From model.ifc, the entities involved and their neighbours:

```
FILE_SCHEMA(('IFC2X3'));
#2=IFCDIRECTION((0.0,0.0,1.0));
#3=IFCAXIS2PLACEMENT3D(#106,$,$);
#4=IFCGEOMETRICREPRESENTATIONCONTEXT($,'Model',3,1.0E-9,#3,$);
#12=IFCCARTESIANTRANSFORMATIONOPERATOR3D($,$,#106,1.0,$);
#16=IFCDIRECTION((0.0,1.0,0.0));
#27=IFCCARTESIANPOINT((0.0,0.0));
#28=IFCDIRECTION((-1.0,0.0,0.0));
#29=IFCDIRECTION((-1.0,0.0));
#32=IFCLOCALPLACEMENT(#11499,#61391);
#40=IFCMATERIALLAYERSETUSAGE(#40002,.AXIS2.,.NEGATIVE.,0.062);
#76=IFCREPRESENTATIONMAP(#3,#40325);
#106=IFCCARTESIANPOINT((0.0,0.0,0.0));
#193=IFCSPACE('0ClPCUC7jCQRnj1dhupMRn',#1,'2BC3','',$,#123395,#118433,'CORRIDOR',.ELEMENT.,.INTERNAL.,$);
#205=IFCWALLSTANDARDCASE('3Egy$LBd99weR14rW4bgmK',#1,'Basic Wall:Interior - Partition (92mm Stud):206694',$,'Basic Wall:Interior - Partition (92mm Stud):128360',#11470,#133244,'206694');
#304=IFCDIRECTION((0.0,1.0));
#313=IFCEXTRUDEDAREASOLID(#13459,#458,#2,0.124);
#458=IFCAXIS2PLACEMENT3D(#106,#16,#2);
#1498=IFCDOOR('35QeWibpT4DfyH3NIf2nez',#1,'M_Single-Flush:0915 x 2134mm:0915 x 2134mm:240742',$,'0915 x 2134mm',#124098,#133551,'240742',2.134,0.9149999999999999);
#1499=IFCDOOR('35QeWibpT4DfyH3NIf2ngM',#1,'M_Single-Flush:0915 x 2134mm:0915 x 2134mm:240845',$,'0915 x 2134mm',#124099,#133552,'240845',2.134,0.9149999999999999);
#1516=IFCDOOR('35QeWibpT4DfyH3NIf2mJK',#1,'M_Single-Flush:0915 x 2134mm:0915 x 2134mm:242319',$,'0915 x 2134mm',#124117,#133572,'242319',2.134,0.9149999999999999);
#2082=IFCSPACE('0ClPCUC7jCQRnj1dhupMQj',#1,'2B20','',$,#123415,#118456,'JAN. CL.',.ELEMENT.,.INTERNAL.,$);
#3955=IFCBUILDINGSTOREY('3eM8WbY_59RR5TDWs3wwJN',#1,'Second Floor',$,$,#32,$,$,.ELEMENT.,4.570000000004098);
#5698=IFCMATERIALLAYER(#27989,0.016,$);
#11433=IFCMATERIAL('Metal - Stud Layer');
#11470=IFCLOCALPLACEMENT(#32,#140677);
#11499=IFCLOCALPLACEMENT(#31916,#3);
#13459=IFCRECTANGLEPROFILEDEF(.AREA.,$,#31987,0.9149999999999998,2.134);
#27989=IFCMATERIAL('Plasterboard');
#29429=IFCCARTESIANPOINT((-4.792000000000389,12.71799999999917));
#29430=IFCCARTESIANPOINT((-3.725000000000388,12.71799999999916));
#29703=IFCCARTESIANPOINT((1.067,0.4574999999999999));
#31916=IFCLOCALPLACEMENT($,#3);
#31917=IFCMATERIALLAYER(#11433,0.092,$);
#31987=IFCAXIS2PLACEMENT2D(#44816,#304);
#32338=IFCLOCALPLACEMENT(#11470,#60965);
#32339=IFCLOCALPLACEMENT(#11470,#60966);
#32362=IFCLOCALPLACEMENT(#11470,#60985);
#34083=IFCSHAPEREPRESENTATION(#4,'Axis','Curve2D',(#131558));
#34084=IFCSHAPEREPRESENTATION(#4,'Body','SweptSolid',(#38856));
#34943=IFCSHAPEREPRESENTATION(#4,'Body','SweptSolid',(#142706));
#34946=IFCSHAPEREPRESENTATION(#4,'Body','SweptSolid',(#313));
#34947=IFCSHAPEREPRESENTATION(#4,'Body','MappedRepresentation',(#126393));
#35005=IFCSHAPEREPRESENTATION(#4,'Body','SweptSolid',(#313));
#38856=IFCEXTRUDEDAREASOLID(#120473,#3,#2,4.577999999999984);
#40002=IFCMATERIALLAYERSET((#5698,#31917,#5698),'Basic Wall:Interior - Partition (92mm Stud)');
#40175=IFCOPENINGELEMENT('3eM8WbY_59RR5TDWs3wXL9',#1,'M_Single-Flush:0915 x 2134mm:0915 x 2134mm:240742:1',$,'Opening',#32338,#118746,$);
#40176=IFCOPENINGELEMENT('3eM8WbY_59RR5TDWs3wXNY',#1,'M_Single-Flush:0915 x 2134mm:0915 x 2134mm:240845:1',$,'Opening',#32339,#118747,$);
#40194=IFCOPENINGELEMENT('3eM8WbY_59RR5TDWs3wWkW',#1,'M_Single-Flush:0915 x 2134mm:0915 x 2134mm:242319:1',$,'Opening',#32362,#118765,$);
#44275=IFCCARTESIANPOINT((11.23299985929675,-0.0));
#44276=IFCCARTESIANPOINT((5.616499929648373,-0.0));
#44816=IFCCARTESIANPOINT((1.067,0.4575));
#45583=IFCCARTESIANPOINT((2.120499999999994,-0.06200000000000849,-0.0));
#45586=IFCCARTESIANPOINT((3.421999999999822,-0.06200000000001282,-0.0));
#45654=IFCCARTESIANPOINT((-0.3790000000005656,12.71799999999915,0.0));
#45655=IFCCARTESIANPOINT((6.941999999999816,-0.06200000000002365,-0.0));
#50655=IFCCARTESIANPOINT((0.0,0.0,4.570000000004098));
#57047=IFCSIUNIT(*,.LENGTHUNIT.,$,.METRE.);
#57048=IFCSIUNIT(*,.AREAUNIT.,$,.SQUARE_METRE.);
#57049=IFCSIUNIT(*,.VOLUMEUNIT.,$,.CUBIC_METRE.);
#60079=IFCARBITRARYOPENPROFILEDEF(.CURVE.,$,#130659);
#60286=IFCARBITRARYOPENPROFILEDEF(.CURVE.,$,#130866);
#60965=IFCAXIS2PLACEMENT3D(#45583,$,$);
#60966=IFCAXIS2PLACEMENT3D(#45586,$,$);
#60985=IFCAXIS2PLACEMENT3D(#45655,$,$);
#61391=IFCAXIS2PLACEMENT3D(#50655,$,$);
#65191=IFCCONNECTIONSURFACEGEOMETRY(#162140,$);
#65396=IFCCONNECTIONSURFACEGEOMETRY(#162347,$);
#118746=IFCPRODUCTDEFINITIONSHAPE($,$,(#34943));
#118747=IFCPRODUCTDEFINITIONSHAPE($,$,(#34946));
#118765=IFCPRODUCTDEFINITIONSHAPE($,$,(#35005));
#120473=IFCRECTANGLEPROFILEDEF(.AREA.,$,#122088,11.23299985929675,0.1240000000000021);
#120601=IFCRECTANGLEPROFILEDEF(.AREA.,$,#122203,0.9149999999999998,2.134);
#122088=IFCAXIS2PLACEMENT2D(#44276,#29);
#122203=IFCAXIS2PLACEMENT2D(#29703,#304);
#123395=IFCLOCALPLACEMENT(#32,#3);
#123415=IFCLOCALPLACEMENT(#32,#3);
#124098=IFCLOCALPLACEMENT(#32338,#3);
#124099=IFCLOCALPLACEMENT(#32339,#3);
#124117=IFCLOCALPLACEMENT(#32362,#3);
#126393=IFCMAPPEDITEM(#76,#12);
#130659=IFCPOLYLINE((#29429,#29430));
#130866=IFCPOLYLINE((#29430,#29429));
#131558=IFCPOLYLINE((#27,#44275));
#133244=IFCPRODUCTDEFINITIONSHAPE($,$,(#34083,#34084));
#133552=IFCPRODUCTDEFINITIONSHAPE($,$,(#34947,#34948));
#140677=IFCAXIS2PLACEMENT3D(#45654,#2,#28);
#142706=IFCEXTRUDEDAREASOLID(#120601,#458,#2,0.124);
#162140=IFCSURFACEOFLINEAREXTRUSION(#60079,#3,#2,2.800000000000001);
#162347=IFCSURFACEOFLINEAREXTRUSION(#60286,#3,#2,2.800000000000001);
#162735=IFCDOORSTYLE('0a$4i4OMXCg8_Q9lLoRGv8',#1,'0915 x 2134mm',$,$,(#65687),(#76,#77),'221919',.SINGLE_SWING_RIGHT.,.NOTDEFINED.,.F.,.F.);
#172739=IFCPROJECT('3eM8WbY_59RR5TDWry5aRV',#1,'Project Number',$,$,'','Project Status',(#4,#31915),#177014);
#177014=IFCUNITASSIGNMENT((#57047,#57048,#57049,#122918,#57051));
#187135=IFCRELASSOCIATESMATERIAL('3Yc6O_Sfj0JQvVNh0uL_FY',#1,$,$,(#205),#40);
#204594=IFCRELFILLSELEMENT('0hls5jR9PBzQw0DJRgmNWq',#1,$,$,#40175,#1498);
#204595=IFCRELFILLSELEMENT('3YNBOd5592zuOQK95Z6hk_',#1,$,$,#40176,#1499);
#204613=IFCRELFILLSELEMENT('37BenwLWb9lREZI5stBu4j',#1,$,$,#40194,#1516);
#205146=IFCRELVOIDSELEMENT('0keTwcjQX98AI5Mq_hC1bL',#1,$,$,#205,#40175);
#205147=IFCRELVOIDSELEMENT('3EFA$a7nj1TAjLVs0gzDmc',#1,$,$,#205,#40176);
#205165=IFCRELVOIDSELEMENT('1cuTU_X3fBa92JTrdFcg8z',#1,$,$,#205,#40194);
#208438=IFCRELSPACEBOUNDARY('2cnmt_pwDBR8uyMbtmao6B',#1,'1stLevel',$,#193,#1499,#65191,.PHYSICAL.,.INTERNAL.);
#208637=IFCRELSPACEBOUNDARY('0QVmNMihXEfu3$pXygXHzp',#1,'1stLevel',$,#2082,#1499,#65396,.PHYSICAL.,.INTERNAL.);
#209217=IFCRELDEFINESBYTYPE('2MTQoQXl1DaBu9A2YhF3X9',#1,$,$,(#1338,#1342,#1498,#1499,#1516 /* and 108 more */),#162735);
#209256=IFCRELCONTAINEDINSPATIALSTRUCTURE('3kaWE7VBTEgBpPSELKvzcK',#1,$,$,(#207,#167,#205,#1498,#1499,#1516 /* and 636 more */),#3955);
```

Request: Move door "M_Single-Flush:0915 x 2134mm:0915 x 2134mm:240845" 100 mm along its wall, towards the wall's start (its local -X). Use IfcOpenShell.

```python
import numpy as np
import ifcopenshell
import ifcopenshell.api.geometry
import ifcopenshell.util.placement
import ifcopenshell.util.unit

model = ifcopenshell.open("model.ifc")
unit_scale = ifcopenshell.util.unit.calculate_unit_scale(model)

door = model.by_guid("35QeWibpT4DfyH3NIf2ngM")
opening = door.FillsVoids[0].RelatingOpeningElement
wall = opening.VoidsElements[0].RelatingBuildingElement

wall_matrix = ifcopenshell.util.placement.get_local_placement(wall.ObjectPlacement)
shift = wall_matrix[:3, 0] * -0.1 / unit_scale
before = ifcopenshell.util.placement.get_local_placement(door.ObjectPlacement)[:3, 3].copy()

# The door is placed relative to its opening, so it follows when the opening moves.
matrix = ifcopenshell.util.placement.get_local_placement(opening.ObjectPlacement)
matrix[:3, 3] += shift
ifcopenshell.api.geometry.edit_object_placement(
    model, product=opening, matrix=matrix, is_si=False, should_transform_children=True
)

# Space boundary surfaces are stored in each space's coordinates; move them too.
for rel in door.ProvidesBoundaries:
    if not rel.ConnectionGeometry:
        continue
    surface = rel.ConnectionGeometry.SurfaceOnRelatingElement
    space_matrix = ifcopenshell.util.placement.get_local_placement(rel.RelatingSpace.ObjectPlacement)
    point = np.array(surface.Position.Location.Coordinates) + space_matrix[:3, :3].T @ shift
    surface.Position = model.createIfcAxis2Placement3D(
        model.createIfcCartesianPoint(point.tolist()), surface.Position.Axis, surface.Position.RefDirection
    )

after = ifcopenshell.util.placement.get_local_placement(door.ObjectPlacement)[:3, 3]
print("door moved by", (after - before).round(3) + 0.0)

model.write("model_edited.ifc")
```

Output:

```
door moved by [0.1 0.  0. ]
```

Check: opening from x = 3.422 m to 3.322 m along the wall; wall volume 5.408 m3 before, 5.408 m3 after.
